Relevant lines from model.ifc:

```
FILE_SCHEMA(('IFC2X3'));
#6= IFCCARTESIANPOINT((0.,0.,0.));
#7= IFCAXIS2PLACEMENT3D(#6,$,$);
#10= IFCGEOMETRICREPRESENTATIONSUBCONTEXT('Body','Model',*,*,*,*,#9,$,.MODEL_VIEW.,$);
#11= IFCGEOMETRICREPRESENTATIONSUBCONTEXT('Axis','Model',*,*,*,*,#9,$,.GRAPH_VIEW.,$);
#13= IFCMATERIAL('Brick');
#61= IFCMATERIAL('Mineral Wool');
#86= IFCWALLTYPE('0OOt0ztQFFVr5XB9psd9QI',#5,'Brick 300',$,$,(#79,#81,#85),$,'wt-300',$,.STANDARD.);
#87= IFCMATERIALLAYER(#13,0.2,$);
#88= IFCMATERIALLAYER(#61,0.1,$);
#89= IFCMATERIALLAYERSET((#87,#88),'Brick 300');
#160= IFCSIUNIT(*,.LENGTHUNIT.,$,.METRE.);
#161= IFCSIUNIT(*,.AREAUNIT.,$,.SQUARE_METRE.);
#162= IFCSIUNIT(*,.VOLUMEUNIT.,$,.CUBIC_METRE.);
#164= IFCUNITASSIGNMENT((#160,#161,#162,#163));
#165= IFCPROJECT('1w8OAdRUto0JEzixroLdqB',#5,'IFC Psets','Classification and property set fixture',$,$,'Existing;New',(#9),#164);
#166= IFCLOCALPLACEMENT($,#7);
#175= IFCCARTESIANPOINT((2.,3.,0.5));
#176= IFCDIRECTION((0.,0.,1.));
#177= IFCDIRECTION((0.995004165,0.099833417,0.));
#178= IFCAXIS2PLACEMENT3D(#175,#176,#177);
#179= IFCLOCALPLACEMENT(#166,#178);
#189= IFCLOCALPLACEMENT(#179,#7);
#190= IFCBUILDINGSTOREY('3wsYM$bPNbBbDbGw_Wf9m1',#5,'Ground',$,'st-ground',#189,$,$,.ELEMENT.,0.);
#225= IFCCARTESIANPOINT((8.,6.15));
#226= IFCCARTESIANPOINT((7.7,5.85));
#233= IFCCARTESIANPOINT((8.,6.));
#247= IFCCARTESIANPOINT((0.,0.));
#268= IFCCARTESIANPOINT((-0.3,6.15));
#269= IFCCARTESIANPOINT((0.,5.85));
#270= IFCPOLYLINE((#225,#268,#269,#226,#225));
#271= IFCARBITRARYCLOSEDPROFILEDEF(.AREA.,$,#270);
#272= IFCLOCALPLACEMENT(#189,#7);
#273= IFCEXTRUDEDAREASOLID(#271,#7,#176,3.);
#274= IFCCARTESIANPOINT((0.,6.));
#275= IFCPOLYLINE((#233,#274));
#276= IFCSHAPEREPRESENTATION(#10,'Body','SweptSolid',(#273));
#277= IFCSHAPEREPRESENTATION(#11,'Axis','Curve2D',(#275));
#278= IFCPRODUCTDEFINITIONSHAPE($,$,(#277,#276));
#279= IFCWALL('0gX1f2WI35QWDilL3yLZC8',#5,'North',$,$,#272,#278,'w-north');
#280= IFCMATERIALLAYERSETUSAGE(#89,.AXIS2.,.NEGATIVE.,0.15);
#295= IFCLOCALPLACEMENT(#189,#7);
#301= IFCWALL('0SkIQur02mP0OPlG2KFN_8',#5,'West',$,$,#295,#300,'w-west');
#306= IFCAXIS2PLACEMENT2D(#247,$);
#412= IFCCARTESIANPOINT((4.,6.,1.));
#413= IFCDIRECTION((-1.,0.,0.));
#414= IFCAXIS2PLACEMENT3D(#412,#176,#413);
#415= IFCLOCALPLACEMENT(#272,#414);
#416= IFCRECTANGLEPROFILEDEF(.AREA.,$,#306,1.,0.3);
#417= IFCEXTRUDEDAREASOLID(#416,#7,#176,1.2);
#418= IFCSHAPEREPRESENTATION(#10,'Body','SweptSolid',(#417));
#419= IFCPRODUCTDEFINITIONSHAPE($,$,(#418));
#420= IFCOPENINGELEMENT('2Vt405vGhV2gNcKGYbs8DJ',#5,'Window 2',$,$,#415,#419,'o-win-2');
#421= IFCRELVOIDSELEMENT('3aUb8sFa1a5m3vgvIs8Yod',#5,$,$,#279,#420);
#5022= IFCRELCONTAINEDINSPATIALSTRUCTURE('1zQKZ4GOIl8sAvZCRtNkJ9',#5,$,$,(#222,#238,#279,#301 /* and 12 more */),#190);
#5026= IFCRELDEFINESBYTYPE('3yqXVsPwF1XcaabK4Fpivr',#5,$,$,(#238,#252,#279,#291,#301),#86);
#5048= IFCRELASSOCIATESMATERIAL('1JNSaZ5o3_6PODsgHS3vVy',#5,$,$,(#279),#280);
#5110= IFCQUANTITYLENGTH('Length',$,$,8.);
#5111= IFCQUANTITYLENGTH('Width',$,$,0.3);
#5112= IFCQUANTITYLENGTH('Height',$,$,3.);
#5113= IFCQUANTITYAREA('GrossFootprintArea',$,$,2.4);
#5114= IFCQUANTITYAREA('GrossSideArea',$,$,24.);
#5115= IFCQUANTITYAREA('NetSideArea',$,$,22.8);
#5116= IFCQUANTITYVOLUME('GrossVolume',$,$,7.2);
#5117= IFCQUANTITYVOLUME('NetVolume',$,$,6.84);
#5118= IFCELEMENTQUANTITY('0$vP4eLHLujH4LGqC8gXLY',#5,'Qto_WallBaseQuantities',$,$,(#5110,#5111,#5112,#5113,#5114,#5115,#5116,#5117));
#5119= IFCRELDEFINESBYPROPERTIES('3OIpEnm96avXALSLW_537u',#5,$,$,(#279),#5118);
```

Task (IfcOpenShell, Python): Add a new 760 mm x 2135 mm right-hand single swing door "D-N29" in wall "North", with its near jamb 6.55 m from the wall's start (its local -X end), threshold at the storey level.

```python
import numpy as np
import ifcopenshell
import ifcopenshell.api.feature
import ifcopenshell.api.geometry
import ifcopenshell.api.pset
import ifcopenshell.api.root
import ifcopenshell.api.spatial
import ifcopenshell.api.type
import ifcopenshell.geom
import ifcopenshell.util.element
import ifcopenshell.util.placement
import ifcopenshell.util.representation
import ifcopenshell.util.shape
import ifcopenshell.util.unit

model = ifcopenshell.open("model.ifc")
unit_scale = ifcopenshell.util.unit.calculate_unit_scale(model)
area_scale = ifcopenshell.util.unit.calculate_unit_scale(model, "AREAUNIT")
volume_scale = ifcopenshell.util.unit.calculate_unit_scale(model, "VOLUMEUNIT")
settings = ifcopenshell.geom.settings()


def volume(element):
    """Net volume in cubic metres, openings subtracted."""
    shape = ifcopenshell.geom.create_shape(settings, element)
    return ifcopenshell.util.shape.get_volume(shape.geometry)


wall = model.by_guid("0gX1f2WI35QWDilL3yLZC8")
storey = ifcopenshell.util.element.get_container(wall, ifc_class="IfcBuildingStorey")
context = ifcopenshell.util.representation.get_context(model, "Model", "Body", "MODEL_VIEW")
before = volume(wall)

width, height, from_end, sill = 0.76, 2.135, 6.55, 0.0  # metres

# The wall runs along its own X axis, and the end named is its -X end.
wall_shape = ifcopenshell.geom.create_shape(settings, wall)
x, y, z = ifcopenshell.util.shape.get_vertices(wall_shape.geometry).T
start = x.min() + from_end
face, thickness = float(y.min()), float(y.max() - y.min())
wall_matrix = ifcopenshell.util.placement.get_local_placement(wall.ObjectPlacement)
level = ifcopenshell.util.placement.get_local_placement(storey.ObjectPlacement)[2, 3]


def in_wall(x, y):
    """Placement at x, y metres in the wall's axes, at sill height."""
    matrix = wall_matrix.copy()
    matrix[:, 3] = wall_matrix @ np.array([x / unit_scale, y / unit_scale, 0.0, 1.0])
    matrix[2, 3] = level + sill / unit_scale
    return matrix


# Opening: a box that overshoots both wall faces by 50 mm.
opening = ifcopenshell.api.root.create_entity(model, ifc_class="IfcOpeningElement")
box = ifcopenshell.api.geometry.add_wall_representation(
    model, context=context, length=width, height=height, thickness=thickness + 0.1
)
ifcopenshell.api.geometry.assign_representation(model, product=opening, representation=box)
ifcopenshell.api.geometry.edit_object_placement(model, product=opening, matrix=in_wall(start, face - 0.05), is_si=False)
ifcopenshell.api.feature.add_feature(model, feature=opening, element=wall)

door = ifcopenshell.api.root.create_entity(model, ifc_class="IfcDoor", name="D-N29")
door.OverallWidth, door.OverallHeight = width / unit_scale, height / unit_scale
body = ifcopenshell.api.geometry.add_door_representation(
    model,
    context=context,
    overall_width=door.OverallWidth,
    overall_height=door.OverallHeight,
    operation_type="SINGLE_SWING_RIGHT",
    lining_properties={"LiningDepth": thickness / unit_scale, "ThresholdDepth": thickness / unit_scale},
)
ifcopenshell.api.geometry.assign_representation(model, product=door, representation=body)
ifcopenshell.api.spatial.assign_container(model, products=[door], relating_structure=storey)
fills = ifcopenshell.api.feature.add_filling(model, opening=opening, element=door)
fills.OwnerHistory = door.OwnerHistory  # required in IFC2X3

# IFC2X3 keeps the operation on the door style.
style = ifcopenshell.api.root.create_entity(model, ifc_class="IfcDoorStyle", name="D-N29")
style.OperationType, style.ConstructionType = "SINGLE_SWING_RIGHT", "NOTDEFINED"
style.ParameterTakesPrecedence = style.Sizeable = False
ifcopenshell.api.type.assign_type(model, related_objects=[door], relating_type=style)

# The lining spans the wall, so the door starts at the wall face.
ifcopenshell.api.geometry.edit_object_placement(model, product=door, matrix=in_wall(start, face), is_si=False)

after = volume(wall)

# Update the wall's stored quantities.
qto = model.by_id(ifcopenshell.util.element.get_pset(wall, "Qto_WallBaseQuantities", should_inherit=False)["id"])
ifcopenshell.api.pset.edit_qto(model, qto=qto, properties={
    "NetSideArea": after / thickness / area_scale,
    "NetVolume": after / volume_scale,
})

print(f"wall volume {before:.3f} -> {after:.3f} m3")

model.write("model-out.ifc")
```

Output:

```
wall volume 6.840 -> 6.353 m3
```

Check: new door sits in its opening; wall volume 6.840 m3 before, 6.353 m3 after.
